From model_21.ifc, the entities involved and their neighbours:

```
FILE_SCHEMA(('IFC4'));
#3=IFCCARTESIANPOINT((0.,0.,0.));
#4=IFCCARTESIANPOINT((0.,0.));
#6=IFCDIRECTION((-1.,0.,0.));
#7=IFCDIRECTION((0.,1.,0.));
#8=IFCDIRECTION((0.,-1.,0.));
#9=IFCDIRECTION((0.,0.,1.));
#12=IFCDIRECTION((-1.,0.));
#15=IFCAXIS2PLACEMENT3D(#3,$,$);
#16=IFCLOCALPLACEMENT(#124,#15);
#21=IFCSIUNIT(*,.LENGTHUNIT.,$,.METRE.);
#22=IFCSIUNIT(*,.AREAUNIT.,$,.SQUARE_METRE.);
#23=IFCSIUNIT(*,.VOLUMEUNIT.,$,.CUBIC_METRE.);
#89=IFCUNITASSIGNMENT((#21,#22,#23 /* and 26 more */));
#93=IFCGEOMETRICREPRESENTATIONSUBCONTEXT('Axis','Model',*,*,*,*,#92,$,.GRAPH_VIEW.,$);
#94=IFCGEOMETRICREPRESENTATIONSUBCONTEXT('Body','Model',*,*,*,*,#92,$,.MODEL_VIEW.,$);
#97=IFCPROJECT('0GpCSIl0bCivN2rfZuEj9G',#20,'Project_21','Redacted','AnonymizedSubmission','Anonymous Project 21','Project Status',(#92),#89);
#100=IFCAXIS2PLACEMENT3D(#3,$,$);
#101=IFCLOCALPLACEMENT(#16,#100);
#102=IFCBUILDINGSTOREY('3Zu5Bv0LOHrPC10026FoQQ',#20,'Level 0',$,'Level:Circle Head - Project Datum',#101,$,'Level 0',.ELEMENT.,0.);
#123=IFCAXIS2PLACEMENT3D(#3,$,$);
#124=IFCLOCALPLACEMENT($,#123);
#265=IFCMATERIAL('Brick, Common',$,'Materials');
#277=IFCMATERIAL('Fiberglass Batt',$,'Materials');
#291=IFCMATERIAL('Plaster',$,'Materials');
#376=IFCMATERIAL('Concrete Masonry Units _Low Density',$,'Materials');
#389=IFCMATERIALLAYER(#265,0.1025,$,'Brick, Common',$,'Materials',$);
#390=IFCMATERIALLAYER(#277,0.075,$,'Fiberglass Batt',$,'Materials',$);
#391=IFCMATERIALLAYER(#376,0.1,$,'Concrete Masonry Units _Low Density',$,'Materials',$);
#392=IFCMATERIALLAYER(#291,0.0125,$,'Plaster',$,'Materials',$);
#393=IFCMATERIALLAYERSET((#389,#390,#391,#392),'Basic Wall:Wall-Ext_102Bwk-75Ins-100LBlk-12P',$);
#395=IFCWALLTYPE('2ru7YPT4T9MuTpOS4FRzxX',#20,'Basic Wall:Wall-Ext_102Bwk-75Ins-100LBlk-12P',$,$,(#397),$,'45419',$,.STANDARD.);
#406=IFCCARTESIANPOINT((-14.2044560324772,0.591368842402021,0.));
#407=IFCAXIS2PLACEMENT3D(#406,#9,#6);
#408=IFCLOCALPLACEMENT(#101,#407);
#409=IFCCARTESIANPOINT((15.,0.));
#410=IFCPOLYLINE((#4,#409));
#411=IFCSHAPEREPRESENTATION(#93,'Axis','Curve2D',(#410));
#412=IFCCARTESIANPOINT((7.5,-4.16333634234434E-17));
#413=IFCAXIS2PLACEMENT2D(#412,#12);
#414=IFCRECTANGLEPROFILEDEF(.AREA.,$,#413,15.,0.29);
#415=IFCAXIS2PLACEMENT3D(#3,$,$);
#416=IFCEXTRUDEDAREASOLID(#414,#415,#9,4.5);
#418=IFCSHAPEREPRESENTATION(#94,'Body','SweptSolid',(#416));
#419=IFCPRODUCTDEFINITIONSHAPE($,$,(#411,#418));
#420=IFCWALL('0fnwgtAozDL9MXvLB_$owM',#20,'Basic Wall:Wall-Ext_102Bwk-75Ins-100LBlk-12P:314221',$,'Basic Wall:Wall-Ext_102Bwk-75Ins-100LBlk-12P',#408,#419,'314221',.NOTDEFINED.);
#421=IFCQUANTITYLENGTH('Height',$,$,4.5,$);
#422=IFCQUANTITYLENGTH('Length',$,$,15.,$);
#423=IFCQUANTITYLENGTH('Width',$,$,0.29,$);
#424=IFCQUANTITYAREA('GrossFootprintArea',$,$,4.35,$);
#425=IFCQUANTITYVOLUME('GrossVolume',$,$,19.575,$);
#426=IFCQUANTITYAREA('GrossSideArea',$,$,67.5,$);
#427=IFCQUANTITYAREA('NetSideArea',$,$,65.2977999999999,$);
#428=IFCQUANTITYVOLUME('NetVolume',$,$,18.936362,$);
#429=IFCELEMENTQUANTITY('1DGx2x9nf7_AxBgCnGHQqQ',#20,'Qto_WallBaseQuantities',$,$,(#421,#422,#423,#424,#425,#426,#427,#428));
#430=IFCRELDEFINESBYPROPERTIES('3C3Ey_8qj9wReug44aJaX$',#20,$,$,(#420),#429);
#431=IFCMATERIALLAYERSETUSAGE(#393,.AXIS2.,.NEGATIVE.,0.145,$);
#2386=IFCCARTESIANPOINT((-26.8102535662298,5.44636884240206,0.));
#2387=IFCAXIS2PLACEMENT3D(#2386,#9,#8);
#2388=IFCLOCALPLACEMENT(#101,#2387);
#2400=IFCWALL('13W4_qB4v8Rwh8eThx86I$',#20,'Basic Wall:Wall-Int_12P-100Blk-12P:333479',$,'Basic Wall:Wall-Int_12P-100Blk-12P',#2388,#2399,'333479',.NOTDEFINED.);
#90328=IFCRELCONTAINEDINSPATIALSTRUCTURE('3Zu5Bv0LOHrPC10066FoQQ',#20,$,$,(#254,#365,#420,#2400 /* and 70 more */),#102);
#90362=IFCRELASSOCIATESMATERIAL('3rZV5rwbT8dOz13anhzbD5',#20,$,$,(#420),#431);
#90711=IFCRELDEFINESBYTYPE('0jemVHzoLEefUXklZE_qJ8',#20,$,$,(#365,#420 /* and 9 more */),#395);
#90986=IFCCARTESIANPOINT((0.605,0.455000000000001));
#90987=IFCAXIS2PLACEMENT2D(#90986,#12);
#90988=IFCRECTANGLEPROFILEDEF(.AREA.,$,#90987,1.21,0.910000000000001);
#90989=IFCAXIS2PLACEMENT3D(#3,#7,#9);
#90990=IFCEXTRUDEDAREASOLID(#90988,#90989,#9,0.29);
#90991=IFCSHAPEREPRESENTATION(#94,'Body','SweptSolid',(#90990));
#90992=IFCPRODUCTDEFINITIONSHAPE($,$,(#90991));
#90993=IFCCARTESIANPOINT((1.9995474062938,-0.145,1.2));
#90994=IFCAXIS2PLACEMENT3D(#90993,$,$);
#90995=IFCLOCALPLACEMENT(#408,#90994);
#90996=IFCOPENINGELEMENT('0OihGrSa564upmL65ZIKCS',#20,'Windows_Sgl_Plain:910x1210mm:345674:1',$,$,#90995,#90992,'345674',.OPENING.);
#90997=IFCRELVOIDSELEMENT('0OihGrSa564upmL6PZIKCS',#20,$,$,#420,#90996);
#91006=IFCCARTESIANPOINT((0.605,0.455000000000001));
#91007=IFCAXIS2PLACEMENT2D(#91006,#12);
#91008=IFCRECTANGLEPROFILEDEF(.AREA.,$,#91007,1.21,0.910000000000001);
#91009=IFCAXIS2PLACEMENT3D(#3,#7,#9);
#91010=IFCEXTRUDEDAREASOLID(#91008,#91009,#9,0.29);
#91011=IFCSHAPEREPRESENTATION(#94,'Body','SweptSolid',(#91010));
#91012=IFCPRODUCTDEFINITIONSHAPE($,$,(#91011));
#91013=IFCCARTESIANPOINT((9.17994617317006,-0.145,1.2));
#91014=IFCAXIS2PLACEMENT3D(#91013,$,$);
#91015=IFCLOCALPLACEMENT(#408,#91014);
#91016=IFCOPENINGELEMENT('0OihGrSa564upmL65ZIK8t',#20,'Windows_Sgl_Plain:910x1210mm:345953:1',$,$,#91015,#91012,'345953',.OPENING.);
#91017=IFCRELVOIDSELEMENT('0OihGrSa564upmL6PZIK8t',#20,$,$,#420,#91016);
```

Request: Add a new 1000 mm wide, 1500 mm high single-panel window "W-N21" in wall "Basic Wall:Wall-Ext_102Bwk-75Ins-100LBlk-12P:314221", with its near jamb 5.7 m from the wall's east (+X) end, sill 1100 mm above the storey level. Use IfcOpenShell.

```python
import numpy as np
import ifcopenshell
import ifcopenshell.api.feature
import ifcopenshell.api.geometry
import ifcopenshell.api.pset
import ifcopenshell.api.root
import ifcopenshell.api.spatial
import ifcopenshell.geom
import ifcopenshell.util.element
import ifcopenshell.util.placement
import ifcopenshell.util.representation
import ifcopenshell.util.shape
import ifcopenshell.util.unit

model = ifcopenshell.open("model_21.ifc")
unit_scale = ifcopenshell.util.unit.calculate_unit_scale(model)
area_scale = ifcopenshell.util.unit.calculate_unit_scale(model, "AREAUNIT")
volume_scale = ifcopenshell.util.unit.calculate_unit_scale(model, "VOLUMEUNIT")
settings = ifcopenshell.geom.settings()


def volume(element):
    """Net volume in cubic metres, openings subtracted."""
    shape = ifcopenshell.geom.create_shape(settings, element)
    return ifcopenshell.util.shape.get_volume(shape.geometry)


wall = model.by_guid("0fnwgtAozDL9MXvLB_$owM")
storey = ifcopenshell.util.element.get_container(wall, ifc_class="IfcBuildingStorey")
context = ifcopenshell.util.representation.get_context(model, "Model", "Body", "MODEL_VIEW")
before = volume(wall)

width, height, from_end, sill = 1, 1.5, 5.7, 1.1  # metres

# The wall runs along its own X axis, and the end named is its -X end.
wall_shape = ifcopenshell.geom.create_shape(settings, wall)
x, y, z = ifcopenshell.util.shape.get_vertices(wall_shape.geometry).T
start = x.min() + from_end
face, thickness = float(y.min()), float(y.max() - y.min())
wall_matrix = ifcopenshell.util.placement.get_local_placement(wall.ObjectPlacement)
level = ifcopenshell.util.placement.get_local_placement(storey.ObjectPlacement)[2, 3]


def in_wall(x, y):
    """Placement at x, y metres in the wall's axes, at sill height."""
    matrix = wall_matrix.copy()
    matrix[:, 3] = wall_matrix @ np.array([x / unit_scale, y / unit_scale, 0.0, 1.0])
    matrix[2, 3] = level + sill / unit_scale
    return matrix


# Opening: a box that overshoots both wall faces by 50 mm.
opening = ifcopenshell.api.root.create_entity(model, ifc_class="IfcOpeningElement", predefined_type="OPENING")
box = ifcopenshell.api.geometry.add_wall_representation(
    model, context=context, length=width, height=height, thickness=thickness + 0.1
)
ifcopenshell.api.geometry.assign_representation(model, product=opening, representation=box)
ifcopenshell.api.geometry.edit_object_placement(model, product=opening, matrix=in_wall(start, face - 0.05), is_si=False)
ifcopenshell.api.feature.add_feature(model, feature=opening, element=wall)

window = ifcopenshell.api.root.create_entity(model, ifc_class="IfcWindow", name="W-N21", predefined_type="WINDOW")
window.OverallWidth, window.OverallHeight = width / unit_scale, height / unit_scale
window.PartitioningType = "SINGLE_PANEL"
body = ifcopenshell.api.geometry.add_window_representation(
    model,
    context=context,
    overall_width=window.OverallWidth,
    overall_height=window.OverallHeight,
    partition_type="SINGLE_PANEL",
)
ifcopenshell.api.geometry.assign_representation(model, product=window, representation=body)
ifcopenshell.api.spatial.assign_container(model, products=[window], relating_structure=storey)
ifcopenshell.api.feature.add_filling(model, opening=opening, element=window)

# Centre the window in the wall's thickness.
ifcopenshell.api.geometry.edit_object_placement(model, product=window, matrix=in_wall(start, face), is_si=False)
window_shape = ifcopenshell.geom.create_shape(settings, window)
depth = ifcopenshell.util.shape.get_vertices(window_shape.geometry)[:, 1]
offset = face + thickness / 2 - (depth.min() + depth.max()) / 2
ifcopenshell.api.geometry.edit_object_placement(model, product=window, matrix=in_wall(start, offset), is_si=False)

after = volume(wall)

# Update the wall's stored quantities.
qto = model.by_id(ifcopenshell.util.element.get_pset(wall, "Qto_WallBaseQuantities", should_inherit=False)["id"])
ifcopenshell.api.pset.edit_qto(model, qto=qto, properties={
    "NetSideArea": after / thickness / area_scale,
    "NetVolume": after / volume_scale,
})

print(f"wall volume {before:.3f} -> {after:.3f} m3")

model.write("model_21_rev.ifc")
```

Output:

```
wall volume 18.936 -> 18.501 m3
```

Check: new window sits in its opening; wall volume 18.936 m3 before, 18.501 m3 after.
